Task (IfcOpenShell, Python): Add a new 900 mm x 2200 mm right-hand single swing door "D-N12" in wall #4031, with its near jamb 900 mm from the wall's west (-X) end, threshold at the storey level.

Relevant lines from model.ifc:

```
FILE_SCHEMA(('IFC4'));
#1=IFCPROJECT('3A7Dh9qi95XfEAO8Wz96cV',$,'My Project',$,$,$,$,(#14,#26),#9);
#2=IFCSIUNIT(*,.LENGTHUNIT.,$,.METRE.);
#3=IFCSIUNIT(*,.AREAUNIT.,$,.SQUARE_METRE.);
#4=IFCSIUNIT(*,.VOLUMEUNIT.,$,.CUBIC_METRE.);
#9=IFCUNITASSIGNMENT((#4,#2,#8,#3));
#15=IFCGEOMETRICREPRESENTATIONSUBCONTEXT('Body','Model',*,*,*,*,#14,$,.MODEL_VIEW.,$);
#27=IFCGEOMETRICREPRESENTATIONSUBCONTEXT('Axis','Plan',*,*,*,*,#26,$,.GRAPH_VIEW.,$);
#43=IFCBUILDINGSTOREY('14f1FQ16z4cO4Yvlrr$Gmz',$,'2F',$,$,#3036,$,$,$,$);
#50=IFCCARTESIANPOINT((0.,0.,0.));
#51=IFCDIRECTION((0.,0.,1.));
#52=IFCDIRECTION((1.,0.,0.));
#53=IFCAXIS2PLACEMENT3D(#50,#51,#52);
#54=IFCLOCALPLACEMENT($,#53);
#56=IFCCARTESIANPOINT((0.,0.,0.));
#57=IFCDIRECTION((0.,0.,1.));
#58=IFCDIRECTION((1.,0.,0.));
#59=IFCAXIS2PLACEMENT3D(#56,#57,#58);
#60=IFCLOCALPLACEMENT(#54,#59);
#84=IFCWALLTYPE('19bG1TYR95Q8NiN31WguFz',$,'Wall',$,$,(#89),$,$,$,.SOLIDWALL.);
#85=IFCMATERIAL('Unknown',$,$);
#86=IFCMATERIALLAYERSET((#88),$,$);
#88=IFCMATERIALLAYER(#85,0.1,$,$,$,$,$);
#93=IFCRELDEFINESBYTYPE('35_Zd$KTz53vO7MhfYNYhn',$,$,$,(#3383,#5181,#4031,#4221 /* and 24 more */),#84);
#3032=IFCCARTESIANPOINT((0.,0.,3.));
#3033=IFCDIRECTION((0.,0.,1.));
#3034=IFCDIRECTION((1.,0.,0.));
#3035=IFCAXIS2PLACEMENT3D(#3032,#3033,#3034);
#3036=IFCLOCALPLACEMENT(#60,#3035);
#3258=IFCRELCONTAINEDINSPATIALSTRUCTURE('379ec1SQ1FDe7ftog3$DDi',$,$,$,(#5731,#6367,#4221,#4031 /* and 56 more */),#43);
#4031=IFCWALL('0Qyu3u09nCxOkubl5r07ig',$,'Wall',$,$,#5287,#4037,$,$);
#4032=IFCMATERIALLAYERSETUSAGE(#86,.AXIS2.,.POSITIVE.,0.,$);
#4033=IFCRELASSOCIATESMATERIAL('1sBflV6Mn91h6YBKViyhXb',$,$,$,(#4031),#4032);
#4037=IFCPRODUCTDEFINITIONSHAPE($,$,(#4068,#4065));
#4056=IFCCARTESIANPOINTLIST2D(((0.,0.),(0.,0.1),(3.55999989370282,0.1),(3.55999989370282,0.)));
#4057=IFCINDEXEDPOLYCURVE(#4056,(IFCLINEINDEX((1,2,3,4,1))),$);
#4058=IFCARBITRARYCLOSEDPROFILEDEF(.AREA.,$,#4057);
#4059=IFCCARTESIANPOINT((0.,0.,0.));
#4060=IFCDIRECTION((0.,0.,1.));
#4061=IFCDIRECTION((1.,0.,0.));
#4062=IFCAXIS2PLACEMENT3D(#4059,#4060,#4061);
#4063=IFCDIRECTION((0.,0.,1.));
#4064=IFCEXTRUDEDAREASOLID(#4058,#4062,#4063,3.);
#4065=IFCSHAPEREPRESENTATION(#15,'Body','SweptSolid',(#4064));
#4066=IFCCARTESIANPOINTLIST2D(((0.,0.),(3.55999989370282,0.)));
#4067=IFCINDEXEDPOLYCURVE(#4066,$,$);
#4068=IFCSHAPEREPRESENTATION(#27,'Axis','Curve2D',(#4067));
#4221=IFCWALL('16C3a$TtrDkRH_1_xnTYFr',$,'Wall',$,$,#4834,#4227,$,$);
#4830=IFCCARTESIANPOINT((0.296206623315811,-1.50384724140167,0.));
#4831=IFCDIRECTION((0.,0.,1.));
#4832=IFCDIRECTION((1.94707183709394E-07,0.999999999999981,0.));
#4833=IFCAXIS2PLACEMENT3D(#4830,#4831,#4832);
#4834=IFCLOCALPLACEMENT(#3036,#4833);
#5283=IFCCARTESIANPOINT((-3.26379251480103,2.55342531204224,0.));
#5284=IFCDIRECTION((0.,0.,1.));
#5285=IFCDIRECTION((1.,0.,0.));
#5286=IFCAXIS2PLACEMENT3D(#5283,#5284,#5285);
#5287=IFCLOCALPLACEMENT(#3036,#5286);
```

```python
import numpy as np
import ifcopenshell
import ifcopenshell.api.feature
import ifcopenshell.api.geometry
import ifcopenshell.api.root
import ifcopenshell.api.spatial
import ifcopenshell.geom
import ifcopenshell.util.element
import ifcopenshell.util.placement
import ifcopenshell.util.representation
import ifcopenshell.util.shape
import ifcopenshell.util.unit

model = ifcopenshell.open("model.ifc")
unit_scale = ifcopenshell.util.unit.calculate_unit_scale(model)
settings = ifcopenshell.geom.settings()


def volume(element):
    """Net volume in cubic metres, openings subtracted."""
    shape = ifcopenshell.geom.create_shape(settings, element)
    return ifcopenshell.util.shape.get_volume(shape.geometry)


wall = model.by_guid("0Qyu3u09nCxOkubl5r07ig")
storey = ifcopenshell.util.element.get_container(wall, ifc_class="IfcBuildingStorey")
context = ifcopenshell.util.representation.get_context(model, "Model", "Body", "MODEL_VIEW")
before = volume(wall)

width, height, from_end, sill = 0.9, 2.2, 0.9, 0.0  # metres

# The wall runs along its own X axis, and the end named is its -X end.
wall_shape = ifcopenshell.geom.create_shape(settings, wall)
x, y, z = ifcopenshell.util.shape.get_vertices(wall_shape.geometry).T
start = x.min() + from_end
face, thickness = float(y.min()), float(y.max() - y.min())
wall_matrix = ifcopenshell.util.placement.get_local_placement(wall.ObjectPlacement)
level = ifcopenshell.util.placement.get_local_placement(storey.ObjectPlacement)[2, 3]


def in_wall(x, y):
    """Placement at x, y metres in the wall's axes, at sill height."""
    matrix = wall_matrix.copy()
    matrix[:, 3] = wall_matrix @ np.array([x / unit_scale, y / unit_scale, 0.0, 1.0])
    matrix[2, 3] = level + sill / unit_scale
    return matrix


# Opening: a box that overshoots both wall faces by 50 mm.
opening = ifcopenshell.api.root.create_entity(model, ifc_class="IfcOpeningElement", predefined_type="OPENING")
box = ifcopenshell.api.geometry.add_wall_representation(
    model, context=context, length=width, height=height, thickness=thickness + 0.1
)
ifcopenshell.api.geometry.assign_representation(model, product=opening, representation=box)
ifcopenshell.api.geometry.edit_object_placement(model, product=opening, matrix=in_wall(start, face - 0.05), is_si=False)
ifcopenshell.api.feature.add_feature(model, feature=opening, element=wall)

door = ifcopenshell.api.root.create_entity(model, ifc_class="IfcDoor", name="D-N12", predefined_type="DOOR")
door.OverallWidth, door.OverallHeight = width / unit_scale, height / unit_scale
door.OperationType = "SINGLE_SWING_RIGHT"
body = ifcopenshell.api.geometry.add_door_representation(
    model,
    context=context,
    overall_width=door.OverallWidth,
    overall_height=door.OverallHeight,
    operation_type="SINGLE_SWING_RIGHT",
    lining_properties={"LiningDepth": thickness / unit_scale, "ThresholdDepth": thickness / unit_scale},
)
ifcopenshell.api.geometry.assign_representation(model, product=door, representation=body)
ifcopenshell.api.spatial.assign_container(model, products=[door], relating_structure=storey)
ifcopenshell.api.feature.add_filling(model, opening=opening, element=door)

# The lining spans the wall, so the door starts at the wall face.
ifcopenshell.api.geometry.edit_object_placement(model, product=door, matrix=in_wall(start, face), is_si=False)

after = volume(wall)

print(f"wall volume {before:.3f} -> {after:.3f} m3")

model.write("model_edited.ifc")
```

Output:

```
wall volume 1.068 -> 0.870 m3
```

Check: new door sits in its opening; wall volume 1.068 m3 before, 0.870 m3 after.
